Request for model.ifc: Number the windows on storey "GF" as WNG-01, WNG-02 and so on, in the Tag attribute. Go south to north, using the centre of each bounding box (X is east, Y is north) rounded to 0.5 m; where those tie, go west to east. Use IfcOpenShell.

First a look at what the model holds.

```python
import ifcopenshell
import ifcopenshell.util.element
import ifcopenshell.util.placement

model = ifcopenshell.open("model.ifc")
print(model.schema)
storey = next(s for s in model.by_type("IfcBuildingStorey") if s.Name == "GF")
windows = [e for e in ifcopenshell.util.element.get_decomposition(storey) if e.is_a("IfcWindow")]
for e in sorted(windows, key=lambda e: e.id()):
    origin = ifcopenshell.util.placement.get_local_placement(e.ObjectPlacement)[:3, 3]
    print(e.id(), e.Tag, e.Name, origin.round(2) + 0.0, sep=" | ")
```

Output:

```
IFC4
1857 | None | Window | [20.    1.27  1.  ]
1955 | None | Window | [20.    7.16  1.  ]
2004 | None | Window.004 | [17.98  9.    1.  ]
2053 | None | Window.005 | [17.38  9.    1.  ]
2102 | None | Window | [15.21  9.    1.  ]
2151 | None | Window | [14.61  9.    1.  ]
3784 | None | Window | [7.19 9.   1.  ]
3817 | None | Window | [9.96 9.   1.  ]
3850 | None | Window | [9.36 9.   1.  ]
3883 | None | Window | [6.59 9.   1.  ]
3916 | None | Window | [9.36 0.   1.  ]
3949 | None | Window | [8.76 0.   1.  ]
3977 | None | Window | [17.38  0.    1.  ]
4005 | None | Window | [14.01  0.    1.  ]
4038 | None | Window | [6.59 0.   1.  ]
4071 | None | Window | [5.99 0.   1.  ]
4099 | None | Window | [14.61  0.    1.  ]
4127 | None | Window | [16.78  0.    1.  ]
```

```python
import ifcopenshell
import ifcopenshell.geom
import ifcopenshell.util.element
import ifcopenshell.util.shape

model = ifcopenshell.open("model.ifc")
settings = ifcopenshell.geom.settings()
settings.set("use-world-coords", True)


def centre(element):
    shape = ifcopenshell.geom.create_shape(settings, element)
    return ifcopenshell.util.shape.get_bbox_centroid(shape.geometry)


storey = next(s for s in model.by_type("IfcBuildingStorey") if s.Name == "GF")
windows = [e for e in ifcopenshell.util.element.get_decomposition(storey) if e.is_a("IfcWindow")]

# Insertion points can sit at a corner or the storey origin, so sort by the geometry (in metres).
centres = {e: centre(e) for e in windows}
windows.sort(key=lambda e: (round(centres[e][1] / 0.5), centres[e][0]))

for i, e in enumerate(windows, start=1):
    number = f"WNG-{i:02d}"
    e.Tag = number
    print(e.id(), number)

model.write("model_edited.ifc")
```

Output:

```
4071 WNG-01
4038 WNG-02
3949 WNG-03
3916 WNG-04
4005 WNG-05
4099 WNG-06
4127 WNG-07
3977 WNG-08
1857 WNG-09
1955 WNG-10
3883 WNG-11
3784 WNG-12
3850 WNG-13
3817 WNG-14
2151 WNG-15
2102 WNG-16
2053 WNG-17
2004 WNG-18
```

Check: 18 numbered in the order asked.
